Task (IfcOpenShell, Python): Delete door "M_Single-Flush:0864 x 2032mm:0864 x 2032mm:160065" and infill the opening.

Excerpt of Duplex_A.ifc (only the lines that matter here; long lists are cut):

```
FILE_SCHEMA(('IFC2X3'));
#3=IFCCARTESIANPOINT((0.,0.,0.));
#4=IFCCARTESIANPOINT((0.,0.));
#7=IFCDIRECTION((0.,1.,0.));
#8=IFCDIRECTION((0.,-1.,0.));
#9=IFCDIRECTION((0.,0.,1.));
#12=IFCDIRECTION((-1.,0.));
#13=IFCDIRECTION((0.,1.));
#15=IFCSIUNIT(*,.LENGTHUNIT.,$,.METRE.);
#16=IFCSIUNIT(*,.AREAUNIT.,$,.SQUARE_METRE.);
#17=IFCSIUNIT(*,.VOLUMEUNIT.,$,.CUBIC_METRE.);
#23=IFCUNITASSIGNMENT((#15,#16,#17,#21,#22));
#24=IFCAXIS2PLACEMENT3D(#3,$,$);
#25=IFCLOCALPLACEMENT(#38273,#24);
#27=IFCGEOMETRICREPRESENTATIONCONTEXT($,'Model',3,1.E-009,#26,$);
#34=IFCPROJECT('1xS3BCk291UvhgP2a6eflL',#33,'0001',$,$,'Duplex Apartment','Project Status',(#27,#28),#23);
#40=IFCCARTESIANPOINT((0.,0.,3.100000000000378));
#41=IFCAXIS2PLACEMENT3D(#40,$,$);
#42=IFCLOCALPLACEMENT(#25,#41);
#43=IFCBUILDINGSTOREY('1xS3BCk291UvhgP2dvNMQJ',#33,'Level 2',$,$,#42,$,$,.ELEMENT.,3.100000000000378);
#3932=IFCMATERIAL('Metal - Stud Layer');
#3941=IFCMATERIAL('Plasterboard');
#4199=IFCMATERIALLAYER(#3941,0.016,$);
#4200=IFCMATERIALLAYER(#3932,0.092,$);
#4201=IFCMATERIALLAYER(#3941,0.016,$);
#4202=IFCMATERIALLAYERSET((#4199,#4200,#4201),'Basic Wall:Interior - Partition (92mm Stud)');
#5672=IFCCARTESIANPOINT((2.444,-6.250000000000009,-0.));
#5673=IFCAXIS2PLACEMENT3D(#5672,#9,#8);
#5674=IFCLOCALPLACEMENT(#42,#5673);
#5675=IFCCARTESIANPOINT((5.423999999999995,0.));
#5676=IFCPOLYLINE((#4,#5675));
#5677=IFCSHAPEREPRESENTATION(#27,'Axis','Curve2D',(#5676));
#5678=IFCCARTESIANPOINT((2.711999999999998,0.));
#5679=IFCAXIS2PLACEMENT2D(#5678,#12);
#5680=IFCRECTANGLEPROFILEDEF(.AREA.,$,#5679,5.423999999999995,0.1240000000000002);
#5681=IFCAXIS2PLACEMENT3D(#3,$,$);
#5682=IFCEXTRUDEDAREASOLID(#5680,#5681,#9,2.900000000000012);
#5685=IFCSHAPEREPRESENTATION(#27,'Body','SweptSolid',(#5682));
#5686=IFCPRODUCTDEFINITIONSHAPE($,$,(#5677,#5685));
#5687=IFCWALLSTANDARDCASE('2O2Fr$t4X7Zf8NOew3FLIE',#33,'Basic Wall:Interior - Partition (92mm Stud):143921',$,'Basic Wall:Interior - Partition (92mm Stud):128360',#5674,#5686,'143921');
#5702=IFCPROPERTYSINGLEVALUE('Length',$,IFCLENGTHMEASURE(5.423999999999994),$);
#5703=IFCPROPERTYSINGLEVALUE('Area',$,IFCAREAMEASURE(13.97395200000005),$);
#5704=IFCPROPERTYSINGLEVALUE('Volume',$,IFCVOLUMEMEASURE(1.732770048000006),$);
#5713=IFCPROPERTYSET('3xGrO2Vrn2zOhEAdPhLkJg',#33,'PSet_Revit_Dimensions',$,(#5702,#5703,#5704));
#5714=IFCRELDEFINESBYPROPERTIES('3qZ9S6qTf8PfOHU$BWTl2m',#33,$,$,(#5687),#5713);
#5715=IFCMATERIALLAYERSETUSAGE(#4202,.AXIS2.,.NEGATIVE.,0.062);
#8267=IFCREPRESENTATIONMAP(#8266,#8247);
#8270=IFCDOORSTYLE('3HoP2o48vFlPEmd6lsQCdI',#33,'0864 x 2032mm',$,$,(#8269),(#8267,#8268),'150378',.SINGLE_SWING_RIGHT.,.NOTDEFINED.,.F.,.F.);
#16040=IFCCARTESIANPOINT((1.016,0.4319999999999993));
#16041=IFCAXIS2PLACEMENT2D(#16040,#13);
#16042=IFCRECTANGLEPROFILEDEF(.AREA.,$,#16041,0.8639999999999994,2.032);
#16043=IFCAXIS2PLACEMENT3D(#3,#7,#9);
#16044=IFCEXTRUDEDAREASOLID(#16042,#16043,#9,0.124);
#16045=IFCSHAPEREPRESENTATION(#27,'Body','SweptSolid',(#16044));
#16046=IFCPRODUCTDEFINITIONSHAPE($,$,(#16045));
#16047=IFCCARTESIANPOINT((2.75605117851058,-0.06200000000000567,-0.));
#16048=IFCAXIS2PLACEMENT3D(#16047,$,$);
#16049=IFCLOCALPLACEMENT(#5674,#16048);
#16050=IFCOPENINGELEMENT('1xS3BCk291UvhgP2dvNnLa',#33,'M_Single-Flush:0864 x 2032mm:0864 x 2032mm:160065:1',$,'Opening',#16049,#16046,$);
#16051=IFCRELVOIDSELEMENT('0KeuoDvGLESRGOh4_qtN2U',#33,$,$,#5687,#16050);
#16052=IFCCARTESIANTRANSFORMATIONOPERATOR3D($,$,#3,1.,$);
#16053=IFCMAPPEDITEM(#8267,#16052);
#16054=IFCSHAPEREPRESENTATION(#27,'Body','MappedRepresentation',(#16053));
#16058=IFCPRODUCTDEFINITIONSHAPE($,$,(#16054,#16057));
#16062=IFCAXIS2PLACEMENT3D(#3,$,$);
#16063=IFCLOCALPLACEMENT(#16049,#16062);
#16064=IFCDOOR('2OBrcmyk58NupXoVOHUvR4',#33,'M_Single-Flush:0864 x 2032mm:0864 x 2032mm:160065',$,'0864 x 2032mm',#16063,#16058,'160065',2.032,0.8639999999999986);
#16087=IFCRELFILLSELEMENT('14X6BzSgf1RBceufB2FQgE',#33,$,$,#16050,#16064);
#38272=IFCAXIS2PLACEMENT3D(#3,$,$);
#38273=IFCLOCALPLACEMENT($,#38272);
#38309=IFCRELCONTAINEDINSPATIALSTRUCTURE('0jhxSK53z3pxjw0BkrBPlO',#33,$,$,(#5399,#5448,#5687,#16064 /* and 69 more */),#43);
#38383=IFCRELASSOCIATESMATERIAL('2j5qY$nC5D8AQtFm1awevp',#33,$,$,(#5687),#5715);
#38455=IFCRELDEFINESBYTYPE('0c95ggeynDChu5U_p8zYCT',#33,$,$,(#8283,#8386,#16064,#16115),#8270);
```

```python
import ifcopenshell
import ifcopenshell.api.feature
import ifcopenshell.api.pset
import ifcopenshell.api.root
import ifcopenshell.geom
import ifcopenshell.util.element
import ifcopenshell.util.shape
import ifcopenshell.util.unit

model = ifcopenshell.open("Duplex_A.ifc")
area_scale = ifcopenshell.util.unit.calculate_unit_scale(model, "AREAUNIT")
volume_scale = ifcopenshell.util.unit.calculate_unit_scale(model, "VOLUMEUNIT")
settings = ifcopenshell.geom.settings()


def volume(element):
    """Net volume in cubic metres, openings subtracted."""
    shape = ifcopenshell.geom.create_shape(settings, element)
    return ifcopenshell.util.shape.get_volume(shape.geometry)


door = model.by_guid("2OBrcmyk58NupXoVOHUvR4")
opening = door.FillsVoids[0].RelatingOpeningElement
wall = opening.VoidsElements[0].RelatingBuildingElement
before = volume(wall)

ifcopenshell.api.root.remove_product(model, product=door)
ifcopenshell.api.feature.remove_feature(model, feature=opening)

after = volume(wall)
thickness = 0.124  # wall thickness in metres

# Update the wall's stored quantities.
pset = model.by_id(ifcopenshell.util.element.get_pset(wall, "PSet_Revit_Dimensions", should_inherit=False)["id"])
ifcopenshell.api.pset.edit_pset(model, pset=pset, properties={
    "Area": model.create_entity("IfcAreaMeasure", after / thickness / area_scale),
    "Volume": model.create_entity("IfcVolumeMeasure", after / volume_scale),
})

print(f"wall volume {before:.3f} -> {after:.3f} m3")

model.write("Duplex_A_updated.ifc")
```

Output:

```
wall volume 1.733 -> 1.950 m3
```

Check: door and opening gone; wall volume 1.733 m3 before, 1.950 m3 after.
